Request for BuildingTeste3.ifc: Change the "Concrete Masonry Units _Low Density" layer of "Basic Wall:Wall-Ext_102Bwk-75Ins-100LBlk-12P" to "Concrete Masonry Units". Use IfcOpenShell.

First a look at what the model holds.

```python
import ifcopenshell
import ifcopenshell.util.element

model = ifcopenshell.open("BuildingTeste3.ifc")
print(model.schema)
for layer_set in model.by_type("IfcMaterialLayerSet"):
    if layer_set.LayerSetName == "Basic Wall:Wall-Ext_102Bwk-75Ins-100LBlk-12P":
        for layer in layer_set.MaterialLayers:
            print(layer.id(), layer.Material and layer.Material.Name, layer.LayerThickness, sep=" | ")
        print(len(ifcopenshell.util.element.get_elements_by_material(model, layer_set)), "elements and types use it")
print(sorted(m.Name for m in model.by_type("IfcMaterial") if m.Name)[:60])
```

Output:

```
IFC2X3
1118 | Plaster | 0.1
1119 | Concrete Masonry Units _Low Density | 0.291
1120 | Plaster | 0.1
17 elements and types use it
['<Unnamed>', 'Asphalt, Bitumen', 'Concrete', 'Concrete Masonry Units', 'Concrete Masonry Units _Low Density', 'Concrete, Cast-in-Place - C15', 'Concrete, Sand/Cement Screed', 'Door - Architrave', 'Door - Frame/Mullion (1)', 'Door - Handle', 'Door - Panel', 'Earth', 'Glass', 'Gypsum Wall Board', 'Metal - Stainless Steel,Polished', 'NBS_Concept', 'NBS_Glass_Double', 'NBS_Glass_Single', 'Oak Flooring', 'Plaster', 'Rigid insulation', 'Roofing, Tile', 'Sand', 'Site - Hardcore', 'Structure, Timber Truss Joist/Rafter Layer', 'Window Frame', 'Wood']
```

```python
import ifcopenshell
import ifcopenshell.api.material

model = ifcopenshell.open("BuildingTeste3.ifc")

layer_set = next(s for s in model.by_type("IfcMaterialLayerSet") if s.LayerSetName == "Basic Wall:Wall-Ext_102Bwk-75Ins-100LBlk-12P")
layer = next(l for l in layer_set.MaterialLayers if l.Material and l.Material.Name == "Concrete Masonry Units _Low Density")
material = next(m for m in model.by_type("IfcMaterial") if m.Name == "Concrete Masonry Units")

# Point this one layer at the other material; renaming the old one would change it everywhere.
ifcopenshell.api.material.edit_layer(model, layer=layer, attributes={}, material=material)

print([l.Material.Name if l.Material else None for l in layer_set.MaterialLayers])

model.write("BuildingTeste3-out.ifc")
```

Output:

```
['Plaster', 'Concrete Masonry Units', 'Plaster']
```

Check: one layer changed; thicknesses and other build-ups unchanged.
